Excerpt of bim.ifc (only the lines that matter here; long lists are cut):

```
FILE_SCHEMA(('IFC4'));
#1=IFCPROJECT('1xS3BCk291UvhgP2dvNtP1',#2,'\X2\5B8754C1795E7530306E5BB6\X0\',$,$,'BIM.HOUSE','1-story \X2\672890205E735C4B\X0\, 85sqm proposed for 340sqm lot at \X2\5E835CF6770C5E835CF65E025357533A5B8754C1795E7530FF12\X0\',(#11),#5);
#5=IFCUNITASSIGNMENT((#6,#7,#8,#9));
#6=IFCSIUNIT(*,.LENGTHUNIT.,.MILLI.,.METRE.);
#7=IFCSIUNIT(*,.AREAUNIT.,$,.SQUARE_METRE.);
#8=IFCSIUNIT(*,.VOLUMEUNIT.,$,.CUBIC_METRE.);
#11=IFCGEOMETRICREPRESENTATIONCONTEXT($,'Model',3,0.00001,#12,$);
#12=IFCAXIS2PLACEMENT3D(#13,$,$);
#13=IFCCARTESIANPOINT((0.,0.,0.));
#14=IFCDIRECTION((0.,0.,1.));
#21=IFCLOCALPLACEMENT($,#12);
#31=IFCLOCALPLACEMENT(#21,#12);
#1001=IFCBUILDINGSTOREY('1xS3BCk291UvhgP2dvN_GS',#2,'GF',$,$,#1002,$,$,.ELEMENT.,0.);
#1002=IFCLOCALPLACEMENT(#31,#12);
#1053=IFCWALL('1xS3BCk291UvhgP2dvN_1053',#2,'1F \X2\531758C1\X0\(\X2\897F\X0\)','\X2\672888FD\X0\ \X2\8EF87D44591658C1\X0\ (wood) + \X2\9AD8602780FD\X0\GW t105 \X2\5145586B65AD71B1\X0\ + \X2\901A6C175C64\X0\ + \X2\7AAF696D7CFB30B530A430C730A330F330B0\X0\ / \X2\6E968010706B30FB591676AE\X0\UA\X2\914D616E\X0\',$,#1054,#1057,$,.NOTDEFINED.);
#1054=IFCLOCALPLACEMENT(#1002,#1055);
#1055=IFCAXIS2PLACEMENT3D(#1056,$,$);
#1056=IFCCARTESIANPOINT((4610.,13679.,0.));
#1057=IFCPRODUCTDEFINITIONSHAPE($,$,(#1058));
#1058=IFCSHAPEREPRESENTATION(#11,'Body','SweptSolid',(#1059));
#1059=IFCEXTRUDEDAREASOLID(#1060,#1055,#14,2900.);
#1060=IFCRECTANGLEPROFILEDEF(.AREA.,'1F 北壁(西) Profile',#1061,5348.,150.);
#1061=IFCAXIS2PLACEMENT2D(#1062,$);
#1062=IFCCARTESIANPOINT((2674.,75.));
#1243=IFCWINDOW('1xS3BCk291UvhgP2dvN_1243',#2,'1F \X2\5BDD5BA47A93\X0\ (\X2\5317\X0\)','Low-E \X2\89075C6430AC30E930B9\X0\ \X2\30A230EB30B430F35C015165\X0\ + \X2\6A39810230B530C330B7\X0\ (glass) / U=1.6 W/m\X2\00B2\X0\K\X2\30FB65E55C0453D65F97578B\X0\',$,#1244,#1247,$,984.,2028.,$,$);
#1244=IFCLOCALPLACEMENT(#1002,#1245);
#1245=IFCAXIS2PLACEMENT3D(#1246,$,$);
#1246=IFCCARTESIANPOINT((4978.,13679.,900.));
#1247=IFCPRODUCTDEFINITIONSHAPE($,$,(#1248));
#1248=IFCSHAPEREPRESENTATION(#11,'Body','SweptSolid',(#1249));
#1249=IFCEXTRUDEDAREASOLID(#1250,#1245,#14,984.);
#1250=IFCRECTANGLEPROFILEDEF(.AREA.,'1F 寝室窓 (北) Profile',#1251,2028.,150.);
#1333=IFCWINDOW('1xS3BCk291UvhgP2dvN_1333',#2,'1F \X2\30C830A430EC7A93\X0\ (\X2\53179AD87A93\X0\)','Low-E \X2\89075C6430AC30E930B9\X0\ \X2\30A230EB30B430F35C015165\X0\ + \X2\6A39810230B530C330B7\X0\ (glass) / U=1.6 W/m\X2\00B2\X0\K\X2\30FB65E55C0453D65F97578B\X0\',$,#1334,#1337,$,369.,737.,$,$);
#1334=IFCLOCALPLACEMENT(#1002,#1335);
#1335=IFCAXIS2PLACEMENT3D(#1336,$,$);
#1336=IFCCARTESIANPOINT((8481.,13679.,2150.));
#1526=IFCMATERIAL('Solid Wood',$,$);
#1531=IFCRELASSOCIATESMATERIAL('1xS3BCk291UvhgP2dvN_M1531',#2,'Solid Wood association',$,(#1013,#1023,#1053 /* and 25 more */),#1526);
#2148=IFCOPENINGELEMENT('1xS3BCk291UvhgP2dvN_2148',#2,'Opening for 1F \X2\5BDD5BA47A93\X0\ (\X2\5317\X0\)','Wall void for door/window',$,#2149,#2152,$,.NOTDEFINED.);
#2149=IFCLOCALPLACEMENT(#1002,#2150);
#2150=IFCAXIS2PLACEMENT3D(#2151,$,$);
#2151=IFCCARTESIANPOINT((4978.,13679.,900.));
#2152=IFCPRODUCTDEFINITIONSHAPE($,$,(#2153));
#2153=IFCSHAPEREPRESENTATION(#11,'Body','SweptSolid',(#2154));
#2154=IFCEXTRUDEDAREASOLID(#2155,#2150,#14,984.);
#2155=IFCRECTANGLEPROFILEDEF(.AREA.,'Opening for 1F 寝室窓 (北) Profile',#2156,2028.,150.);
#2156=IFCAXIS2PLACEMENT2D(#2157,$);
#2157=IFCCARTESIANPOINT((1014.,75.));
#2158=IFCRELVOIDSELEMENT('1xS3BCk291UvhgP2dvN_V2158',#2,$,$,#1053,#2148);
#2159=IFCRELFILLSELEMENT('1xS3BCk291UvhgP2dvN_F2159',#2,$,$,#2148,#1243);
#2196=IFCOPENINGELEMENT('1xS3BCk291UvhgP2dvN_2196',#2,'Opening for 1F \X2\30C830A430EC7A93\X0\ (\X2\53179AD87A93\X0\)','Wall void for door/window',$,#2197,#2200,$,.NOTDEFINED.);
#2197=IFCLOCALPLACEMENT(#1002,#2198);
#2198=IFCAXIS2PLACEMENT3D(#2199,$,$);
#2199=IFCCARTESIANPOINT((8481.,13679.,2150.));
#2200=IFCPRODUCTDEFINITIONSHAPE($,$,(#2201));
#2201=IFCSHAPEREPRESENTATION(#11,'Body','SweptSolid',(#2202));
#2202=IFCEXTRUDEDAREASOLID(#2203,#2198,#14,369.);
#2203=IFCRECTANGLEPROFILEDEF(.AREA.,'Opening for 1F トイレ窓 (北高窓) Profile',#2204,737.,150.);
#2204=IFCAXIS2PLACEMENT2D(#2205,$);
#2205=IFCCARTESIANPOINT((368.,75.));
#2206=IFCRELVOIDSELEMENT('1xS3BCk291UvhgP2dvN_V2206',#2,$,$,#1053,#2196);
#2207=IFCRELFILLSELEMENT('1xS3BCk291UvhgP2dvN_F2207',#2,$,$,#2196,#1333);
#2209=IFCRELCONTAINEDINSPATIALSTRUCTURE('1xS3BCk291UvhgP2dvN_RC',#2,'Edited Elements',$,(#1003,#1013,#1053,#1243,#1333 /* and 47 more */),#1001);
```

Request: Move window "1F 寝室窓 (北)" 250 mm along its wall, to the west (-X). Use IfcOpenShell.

```python
import ifcopenshell
import ifcopenshell.api.geometry
import ifcopenshell.util.placement

model = ifcopenshell.open("bim.ifc")

window = model.by_guid("1xS3BCk291UvhgP2dvN_1243")
opening = window.FillsVoids[0].RelatingOpeningElement
wall = opening.VoidsElements[0].RelatingBuildingElement

wall_matrix = ifcopenshell.util.placement.get_local_placement(wall.ObjectPlacement)
shift = wall_matrix[:3, 0] * -250.0
before = ifcopenshell.util.placement.get_local_placement(window.ObjectPlacement)[:3, 3].copy()

# The window is not placed relative to its opening, so move both.
for product in (opening, window):
    matrix = ifcopenshell.util.placement.get_local_placement(product.ObjectPlacement)
    matrix[:3, 3] += shift
    ifcopenshell.api.geometry.edit_object_placement(model, product=product, matrix=matrix, is_si=False)

after = ifcopenshell.util.placement.get_local_placement(window.ObjectPlacement)[:3, 3]
print("window moved by", (after - before).round(3) + 0.0)

model.write("bim_edited.ifc")
```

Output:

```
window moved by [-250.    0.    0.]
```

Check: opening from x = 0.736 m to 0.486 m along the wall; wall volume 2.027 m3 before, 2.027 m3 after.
